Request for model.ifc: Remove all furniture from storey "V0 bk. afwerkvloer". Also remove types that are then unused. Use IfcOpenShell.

First a look at what the model holds.

```python
import ifcopenshell
import ifcopenshell.util.element

model = ifcopenshell.open("model.ifc")
print(model.schema)
storey = next(s for s in model.by_type("IfcBuildingStorey") if s.Name == "V0 bk. afwerkvloer")
furniture = [e for e in ifcopenshell.util.element.get_decomposition(storey) if e.is_a("IfcFurnishingElement")]
seen = {}
for e in furniture:
    element_type = ifcopenshell.util.element.get_type(e)
    name = element_type.Name if element_type not in (None, e) else None
    seen[name] = seen.get(name, 0) + 1
for name, count in sorted(seen.items(), key=str):
    print(count, "x", name)
```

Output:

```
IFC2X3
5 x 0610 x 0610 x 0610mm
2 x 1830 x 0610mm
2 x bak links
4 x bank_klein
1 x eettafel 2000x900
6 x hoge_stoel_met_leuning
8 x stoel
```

```python
import ifcopenshell
import ifcopenshell.api.root
import ifcopenshell.util.element

model = ifcopenshell.open("model.ifc")

storey = next(s for s in model.by_type("IfcBuildingStorey") if s.Name == "V0 bk. afwerkvloer")
furniture = [e for e in ifcopenshell.util.element.get_decomposition(storey) if e.is_a("IfcFurnishingElement")]
types = {ifcopenshell.util.element.get_type(e) for e in furniture} - {None, *furniture}

for e in furniture:
    ifcopenshell.api.root.remove_product(model, product=e)
print(len(furniture), "removed")

unused = [t for t in types if not ifcopenshell.util.element.get_types(t)]
for t in unused:
    ifcopenshell.api.root.remove_product(model, product=t)
print(len(unused), "unused types removed")

model.write("model_rev.ifc")
```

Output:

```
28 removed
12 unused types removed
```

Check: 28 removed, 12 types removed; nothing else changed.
